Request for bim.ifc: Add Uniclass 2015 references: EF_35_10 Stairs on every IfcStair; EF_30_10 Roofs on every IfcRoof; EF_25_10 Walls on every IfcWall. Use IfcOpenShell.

First a look at what the model holds.

```python
import ifcopenshell

model = ifcopenshell.open("bim.ifc")
print(model.schema)
print("classifications:", [c.Name for c in model.by_type("IfcClassification")])
for ifc_class in ("IfcDoor", "IfcRoof", "IfcStair", "IfcWall", "IfcWindow"):
    print(ifc_class, len(model.by_type(ifc_class)))
```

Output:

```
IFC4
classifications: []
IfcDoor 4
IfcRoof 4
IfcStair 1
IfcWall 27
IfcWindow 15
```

```python
import ifcopenshell
import ifcopenshell.api.classification

model = ifcopenshell.open("bim.ifc")

system = ifcopenshell.api.classification.add_classification(model, classification="Uniclass 2015")

codes = {
    "IfcStair": ("EF_35_10", "Stairs"),
    "IfcRoof": ("EF_30_10", "Roofs"),
    "IfcWall": ("EF_25_10", "Walls"),
}
for ifc_class, (code, name) in codes.items():
    products = model.by_type(ifc_class)
    ifcopenshell.api.classification.add_reference(
        model, products=products, classification=system, identification=code, name=name
    )
    print(code, len(products))

model.write("bim_rev.ifc")
```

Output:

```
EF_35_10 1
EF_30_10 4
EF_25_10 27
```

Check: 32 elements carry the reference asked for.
